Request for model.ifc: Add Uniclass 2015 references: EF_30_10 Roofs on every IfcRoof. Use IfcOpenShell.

First a look at what the model holds.

```python
import ifcopenshell

model = ifcopenshell.open("model.ifc")
print(model.schema)
print("classifications:", [c.Name for c in model.by_type("IfcClassification")])
for ifc_class in ("IfcDoor", "IfcRoof", "IfcStair", "IfcWall", "IfcWindow"):
    print(ifc_class, len(model.by_type(ifc_class)))
```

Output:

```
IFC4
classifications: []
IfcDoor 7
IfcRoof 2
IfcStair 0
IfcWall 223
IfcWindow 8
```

```python
import ifcopenshell
import ifcopenshell.api.classification

model = ifcopenshell.open("model.ifc")

system = ifcopenshell.api.classification.add_classification(model, classification="Uniclass 2015")

codes = {
    "IfcRoof": ("EF_30_10", "Roofs"),
}
for ifc_class, (code, name) in codes.items():
    products = model.by_type(ifc_class)
    ifcopenshell.api.classification.add_reference(
        model, products=products, classification=system, identification=code, name=name
    )
    print(code, len(products))

model.write("model_v2.ifc")
```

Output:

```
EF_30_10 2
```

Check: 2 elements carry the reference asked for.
